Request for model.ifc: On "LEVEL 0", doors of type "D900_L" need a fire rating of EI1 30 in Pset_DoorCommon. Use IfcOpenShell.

First a look at what the model holds.

```python
import ifcopenshell
import ifcopenshell.util.element

model = ifcopenshell.open("model.ifc")
print(model.schema)
storey = next(s for s in model.by_type("IfcBuildingStorey") if s.Name == "LEVEL 0")
doors = [e for e in ifcopenshell.util.element.get_decomposition(storey) if e.is_a("IfcDoor")]
seen = {}
for e in doors:
    element_type = ifcopenshell.util.element.get_type(e)
    key = (element_type.Name if element_type != e and element_type else None, ifcopenshell.util.element.get_pset(e, "Pset_DoorCommon", "FireRating"))
    seen[key] = seen.get(key, 0) + 1
for (name, value), count in sorted(seen.items(), key=str):
    print(count, "x", name, "|", value)
```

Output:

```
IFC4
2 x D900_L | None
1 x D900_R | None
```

```python
import ifcopenshell
import ifcopenshell.api.pset
import ifcopenshell.util.element

model = ifcopenshell.open("model.ifc")

storey = next(s for s in model.by_type("IfcBuildingStorey") if s.Name == "LEVEL 0")
doors = [e for e in ifcopenshell.util.element.get_decomposition(storey) if e.is_a("IfcDoor")]

count = 0
for e in doors:
    element_type = ifcopenshell.util.element.get_type(e)
    if element_type in (None, e) or element_type.Name != "D900_L":
        continue
    # add_pset returns the element's existing set when there is one.
    pset = ifcopenshell.api.pset.add_pset(model, product=e, name="Pset_DoorCommon")
    ifcopenshell.api.pset.edit_pset(model, pset=pset, properties={"FireRating": "EI1 30"})
    count += 1

print(count, "doors updated")

model.write("model_updated.ifc")
```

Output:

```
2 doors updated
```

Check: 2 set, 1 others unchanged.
